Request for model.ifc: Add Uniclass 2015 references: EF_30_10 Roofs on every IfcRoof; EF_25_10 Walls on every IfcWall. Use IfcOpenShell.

First a look at what the model holds.

```python
import ifcopenshell

model = ifcopenshell.open("model.ifc")
print(model.schema)
print("classifications:", [c.Name for c in model.by_type("IfcClassification")])
for ifc_class in ("IfcDoor", "IfcRoof", "IfcStair", "IfcWall", "IfcWindow"):
    print(ifc_class, len(model.by_type(ifc_class)))
```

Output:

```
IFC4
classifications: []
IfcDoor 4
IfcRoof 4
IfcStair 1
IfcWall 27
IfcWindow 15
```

```python
import ifcopenshell
import ifcopenshell.api.classification

model = ifcopenshell.open("model.ifc")

system = ifcopenshell.api.classification.add_classification(model, classification="Uniclass 2015")

codes = {
    "IfcRoof": ("EF_30_10", "Roofs"),
    "IfcWall": ("EF_25_10", "Walls"),
}
for ifc_class, (code, name) in codes.items():
    products = model.by_type(ifc_class)
    ifcopenshell.api.classification.add_reference(
        model, products=products, classification=system, identification=code, name=name
    )
    print(code, len(products))

model.write("model_rev.ifc")
```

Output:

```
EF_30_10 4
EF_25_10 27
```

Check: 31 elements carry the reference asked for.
